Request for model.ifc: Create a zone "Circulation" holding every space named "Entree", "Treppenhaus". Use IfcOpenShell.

First a look at what the model holds.

```python
import ifcopenshell

model = ifcopenshell.open("model.ifc")
print(model.schema)
seen = {}
for space in model.by_type("IfcSpace"):
    seen[space.LongName] = seen.get(space.LongName, 0) + 1
for name, count in sorted(seen.items(), key=str):
    print(count, "x", name)
print("zones:", [z.Name for z in model.by_type("IfcZone")][:20])
```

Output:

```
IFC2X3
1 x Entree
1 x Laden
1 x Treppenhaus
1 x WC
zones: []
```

```python
import ifcopenshell
import ifcopenshell.api.group
import ifcopenshell.api.root

model = ifcopenshell.open("model.ifc")

names = {"Entree", "Treppenhaus"}
spaces = [s for s in model.by_type("IfcSpace") if s.LongName in names]

zone = ifcopenshell.api.root.create_entity(model, ifc_class="IfcZone", name="Circulation")
ifcopenshell.api.group.assign_group(model, products=spaces, group=zone)
print(len(spaces), "spaces in", zone.Name)

model.write("model_edited.ifc")
```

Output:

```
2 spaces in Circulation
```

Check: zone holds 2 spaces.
